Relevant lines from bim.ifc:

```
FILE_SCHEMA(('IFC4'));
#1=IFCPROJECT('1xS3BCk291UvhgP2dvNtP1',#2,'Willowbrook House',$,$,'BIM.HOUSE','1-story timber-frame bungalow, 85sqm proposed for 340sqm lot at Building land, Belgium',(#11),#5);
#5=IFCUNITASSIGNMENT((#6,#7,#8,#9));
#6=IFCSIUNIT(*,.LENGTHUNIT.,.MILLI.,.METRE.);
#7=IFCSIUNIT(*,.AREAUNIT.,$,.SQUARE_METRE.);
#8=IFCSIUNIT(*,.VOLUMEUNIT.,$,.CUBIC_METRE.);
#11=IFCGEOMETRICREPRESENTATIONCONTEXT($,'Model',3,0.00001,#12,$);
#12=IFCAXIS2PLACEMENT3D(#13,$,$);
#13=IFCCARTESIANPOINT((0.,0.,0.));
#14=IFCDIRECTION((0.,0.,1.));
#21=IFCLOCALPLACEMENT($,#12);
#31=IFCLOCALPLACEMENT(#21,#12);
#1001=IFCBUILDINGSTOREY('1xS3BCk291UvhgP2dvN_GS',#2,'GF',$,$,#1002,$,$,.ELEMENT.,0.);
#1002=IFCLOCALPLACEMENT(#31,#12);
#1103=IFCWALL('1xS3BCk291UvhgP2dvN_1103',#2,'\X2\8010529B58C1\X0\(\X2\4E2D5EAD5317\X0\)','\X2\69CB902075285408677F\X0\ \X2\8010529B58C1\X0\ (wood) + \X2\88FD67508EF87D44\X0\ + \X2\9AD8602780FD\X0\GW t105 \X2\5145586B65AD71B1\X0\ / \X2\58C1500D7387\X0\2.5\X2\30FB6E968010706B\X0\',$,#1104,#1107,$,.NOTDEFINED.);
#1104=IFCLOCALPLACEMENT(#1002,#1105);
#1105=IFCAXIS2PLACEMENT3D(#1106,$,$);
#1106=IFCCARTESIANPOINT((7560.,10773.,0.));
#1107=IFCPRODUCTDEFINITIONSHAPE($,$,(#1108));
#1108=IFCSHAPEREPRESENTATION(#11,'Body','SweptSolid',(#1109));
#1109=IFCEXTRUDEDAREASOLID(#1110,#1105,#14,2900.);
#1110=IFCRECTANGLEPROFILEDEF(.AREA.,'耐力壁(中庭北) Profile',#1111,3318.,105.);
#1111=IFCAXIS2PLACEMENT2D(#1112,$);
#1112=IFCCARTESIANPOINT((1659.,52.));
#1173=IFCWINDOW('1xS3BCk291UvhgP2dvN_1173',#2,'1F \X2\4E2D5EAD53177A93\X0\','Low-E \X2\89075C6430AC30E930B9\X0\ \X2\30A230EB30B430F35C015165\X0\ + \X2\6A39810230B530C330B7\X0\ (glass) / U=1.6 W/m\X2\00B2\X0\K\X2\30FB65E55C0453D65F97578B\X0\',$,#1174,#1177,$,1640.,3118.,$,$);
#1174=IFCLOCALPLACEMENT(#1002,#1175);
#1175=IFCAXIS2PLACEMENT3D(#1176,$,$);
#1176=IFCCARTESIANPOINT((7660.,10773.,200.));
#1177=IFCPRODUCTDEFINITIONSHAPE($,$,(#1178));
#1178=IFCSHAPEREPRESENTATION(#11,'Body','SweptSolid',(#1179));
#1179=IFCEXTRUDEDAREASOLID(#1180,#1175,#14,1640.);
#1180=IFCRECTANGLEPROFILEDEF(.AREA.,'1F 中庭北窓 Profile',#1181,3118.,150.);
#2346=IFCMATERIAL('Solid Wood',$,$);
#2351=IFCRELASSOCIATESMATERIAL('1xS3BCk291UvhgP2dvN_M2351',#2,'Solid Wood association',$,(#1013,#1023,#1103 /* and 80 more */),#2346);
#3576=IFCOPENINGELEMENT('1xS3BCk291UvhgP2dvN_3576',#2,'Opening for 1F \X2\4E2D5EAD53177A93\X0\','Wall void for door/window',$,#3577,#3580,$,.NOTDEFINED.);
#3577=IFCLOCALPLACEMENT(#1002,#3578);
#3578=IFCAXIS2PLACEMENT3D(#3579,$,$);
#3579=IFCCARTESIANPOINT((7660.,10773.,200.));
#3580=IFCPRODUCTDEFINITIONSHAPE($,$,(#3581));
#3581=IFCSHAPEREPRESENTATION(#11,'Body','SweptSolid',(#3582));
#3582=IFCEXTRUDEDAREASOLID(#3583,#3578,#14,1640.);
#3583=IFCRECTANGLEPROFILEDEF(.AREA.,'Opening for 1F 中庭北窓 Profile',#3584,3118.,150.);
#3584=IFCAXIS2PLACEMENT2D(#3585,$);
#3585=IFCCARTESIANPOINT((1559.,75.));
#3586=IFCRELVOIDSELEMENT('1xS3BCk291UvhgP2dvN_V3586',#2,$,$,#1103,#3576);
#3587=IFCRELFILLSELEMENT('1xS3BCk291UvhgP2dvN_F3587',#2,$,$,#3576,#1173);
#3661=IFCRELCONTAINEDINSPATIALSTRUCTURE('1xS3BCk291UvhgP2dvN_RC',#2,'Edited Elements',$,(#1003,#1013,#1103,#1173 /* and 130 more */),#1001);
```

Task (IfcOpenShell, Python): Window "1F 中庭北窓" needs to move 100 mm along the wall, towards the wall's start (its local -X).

```python
import ifcopenshell
import ifcopenshell.api.geometry
import ifcopenshell.util.placement
import ifcopenshell.util.unit

model = ifcopenshell.open("bim.ifc")
unit_scale = ifcopenshell.util.unit.calculate_unit_scale(model)

window = model.by_guid("1xS3BCk291UvhgP2dvN_1173")
opening = window.FillsVoids[0].RelatingOpeningElement
wall = opening.VoidsElements[0].RelatingBuildingElement

wall_matrix = ifcopenshell.util.placement.get_local_placement(wall.ObjectPlacement)
shift = wall_matrix[:3, 0] * -0.1 / unit_scale
before = ifcopenshell.util.placement.get_local_placement(window.ObjectPlacement)[:3, 3].copy()

# The window is not placed relative to its opening, so move both.
for product in (opening, window):
    matrix = ifcopenshell.util.placement.get_local_placement(product.ObjectPlacement)
    matrix[:3, 3] += shift
    ifcopenshell.api.geometry.edit_object_placement(model, product=product, matrix=matrix, is_si=False)

after = ifcopenshell.util.placement.get_local_placement(window.ObjectPlacement)[:3, 3]
print("window moved by", (after - before).round(3) + 0.0)

model.write("bim_rev.ifc")
```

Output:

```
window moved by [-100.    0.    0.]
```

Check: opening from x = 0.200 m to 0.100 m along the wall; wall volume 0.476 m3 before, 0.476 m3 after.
